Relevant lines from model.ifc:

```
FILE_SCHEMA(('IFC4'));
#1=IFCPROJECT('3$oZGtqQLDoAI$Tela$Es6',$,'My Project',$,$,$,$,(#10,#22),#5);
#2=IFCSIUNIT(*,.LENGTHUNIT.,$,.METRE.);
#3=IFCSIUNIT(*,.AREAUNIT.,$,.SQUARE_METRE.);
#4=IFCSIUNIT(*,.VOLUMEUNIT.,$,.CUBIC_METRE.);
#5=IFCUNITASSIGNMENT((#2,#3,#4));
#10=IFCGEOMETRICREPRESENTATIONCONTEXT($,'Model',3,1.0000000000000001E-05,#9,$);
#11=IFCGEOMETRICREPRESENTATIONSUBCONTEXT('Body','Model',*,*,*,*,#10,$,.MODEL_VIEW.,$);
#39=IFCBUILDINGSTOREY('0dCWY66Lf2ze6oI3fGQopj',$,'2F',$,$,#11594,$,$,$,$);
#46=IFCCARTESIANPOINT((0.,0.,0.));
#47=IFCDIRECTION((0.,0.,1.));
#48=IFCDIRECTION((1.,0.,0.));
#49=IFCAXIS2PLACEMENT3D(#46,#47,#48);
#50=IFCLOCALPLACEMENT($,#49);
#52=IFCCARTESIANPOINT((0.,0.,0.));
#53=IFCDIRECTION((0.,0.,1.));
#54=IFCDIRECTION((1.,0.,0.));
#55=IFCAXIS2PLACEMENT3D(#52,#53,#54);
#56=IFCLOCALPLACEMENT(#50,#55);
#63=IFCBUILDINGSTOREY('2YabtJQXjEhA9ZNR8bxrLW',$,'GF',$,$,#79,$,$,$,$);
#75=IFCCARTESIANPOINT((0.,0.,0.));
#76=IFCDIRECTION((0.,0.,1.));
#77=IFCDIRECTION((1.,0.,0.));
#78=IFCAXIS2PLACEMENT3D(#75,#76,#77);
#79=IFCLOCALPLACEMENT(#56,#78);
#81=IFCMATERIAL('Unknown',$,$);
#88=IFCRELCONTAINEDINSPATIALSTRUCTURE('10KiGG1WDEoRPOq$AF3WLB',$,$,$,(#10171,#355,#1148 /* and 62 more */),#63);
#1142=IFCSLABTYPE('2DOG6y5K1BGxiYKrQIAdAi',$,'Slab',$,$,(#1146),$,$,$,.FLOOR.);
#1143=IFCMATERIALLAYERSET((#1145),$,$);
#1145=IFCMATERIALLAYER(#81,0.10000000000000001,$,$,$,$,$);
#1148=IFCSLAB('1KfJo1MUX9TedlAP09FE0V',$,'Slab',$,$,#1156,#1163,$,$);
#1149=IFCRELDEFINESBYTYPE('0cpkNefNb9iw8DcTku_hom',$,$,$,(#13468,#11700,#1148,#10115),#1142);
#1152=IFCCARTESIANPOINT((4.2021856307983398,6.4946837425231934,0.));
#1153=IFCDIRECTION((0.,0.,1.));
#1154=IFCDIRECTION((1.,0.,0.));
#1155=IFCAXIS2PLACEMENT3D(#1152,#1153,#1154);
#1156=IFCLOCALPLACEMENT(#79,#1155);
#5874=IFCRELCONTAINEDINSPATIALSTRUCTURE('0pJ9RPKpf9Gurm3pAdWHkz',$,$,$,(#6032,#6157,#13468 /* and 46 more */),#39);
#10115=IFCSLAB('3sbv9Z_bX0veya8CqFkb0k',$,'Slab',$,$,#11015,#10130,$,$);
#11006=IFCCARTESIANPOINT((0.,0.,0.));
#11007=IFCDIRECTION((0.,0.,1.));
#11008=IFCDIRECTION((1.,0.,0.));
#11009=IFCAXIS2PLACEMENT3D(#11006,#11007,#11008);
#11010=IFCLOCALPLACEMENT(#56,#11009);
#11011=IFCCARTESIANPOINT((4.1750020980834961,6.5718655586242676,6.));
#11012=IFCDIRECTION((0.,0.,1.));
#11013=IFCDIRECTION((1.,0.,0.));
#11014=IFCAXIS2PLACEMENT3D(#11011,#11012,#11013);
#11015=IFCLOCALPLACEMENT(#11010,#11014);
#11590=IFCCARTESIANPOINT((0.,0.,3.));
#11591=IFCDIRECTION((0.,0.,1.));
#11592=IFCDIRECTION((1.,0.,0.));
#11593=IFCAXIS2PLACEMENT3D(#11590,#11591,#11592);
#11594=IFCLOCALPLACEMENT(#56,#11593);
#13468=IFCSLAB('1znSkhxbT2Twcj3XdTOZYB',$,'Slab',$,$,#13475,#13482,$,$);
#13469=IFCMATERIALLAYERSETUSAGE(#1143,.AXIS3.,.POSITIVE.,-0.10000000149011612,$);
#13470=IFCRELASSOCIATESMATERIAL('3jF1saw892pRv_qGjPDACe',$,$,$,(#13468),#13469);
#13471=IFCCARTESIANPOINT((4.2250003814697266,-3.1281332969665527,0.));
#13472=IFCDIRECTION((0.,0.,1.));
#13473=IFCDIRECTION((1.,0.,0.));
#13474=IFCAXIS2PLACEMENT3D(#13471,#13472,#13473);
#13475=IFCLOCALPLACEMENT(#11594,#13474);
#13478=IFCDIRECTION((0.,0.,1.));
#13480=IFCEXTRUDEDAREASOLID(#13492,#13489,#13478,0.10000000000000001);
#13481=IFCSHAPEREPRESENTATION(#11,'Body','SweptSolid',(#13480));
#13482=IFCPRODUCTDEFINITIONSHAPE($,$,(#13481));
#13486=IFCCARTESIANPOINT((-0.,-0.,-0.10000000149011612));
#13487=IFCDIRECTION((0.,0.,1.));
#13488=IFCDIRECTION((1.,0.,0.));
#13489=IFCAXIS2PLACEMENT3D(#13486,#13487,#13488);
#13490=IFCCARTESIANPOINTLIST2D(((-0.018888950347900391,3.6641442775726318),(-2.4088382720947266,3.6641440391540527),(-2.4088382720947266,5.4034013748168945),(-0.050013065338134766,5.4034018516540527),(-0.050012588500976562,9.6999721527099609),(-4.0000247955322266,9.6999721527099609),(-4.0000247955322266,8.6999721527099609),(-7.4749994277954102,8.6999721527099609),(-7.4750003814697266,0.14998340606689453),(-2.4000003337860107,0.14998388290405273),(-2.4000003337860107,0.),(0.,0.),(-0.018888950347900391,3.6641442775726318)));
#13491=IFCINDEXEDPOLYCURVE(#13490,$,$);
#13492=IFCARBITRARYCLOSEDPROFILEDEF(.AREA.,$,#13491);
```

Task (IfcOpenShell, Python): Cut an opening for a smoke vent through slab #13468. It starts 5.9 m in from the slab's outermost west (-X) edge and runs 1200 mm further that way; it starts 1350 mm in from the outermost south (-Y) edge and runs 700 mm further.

```python
import numpy as np
import ifcopenshell
import ifcopenshell.api.feature
import ifcopenshell.api.geometry
import ifcopenshell.api.root
import ifcopenshell.geom
import ifcopenshell.util.placement
import ifcopenshell.util.representation
import ifcopenshell.util.shape
import ifcopenshell.util.unit

model = ifcopenshell.open("model.ifc")
unit_scale = ifcopenshell.util.unit.calculate_unit_scale(model)
settings = ifcopenshell.geom.settings()


def volume(element):
    """Net volume in cubic metres, openings subtracted."""
    shape = ifcopenshell.geom.create_shape(settings, element)
    return ifcopenshell.util.shape.get_volume(shape.geometry)


slab = model.by_guid("1znSkhxbT2Twcj3XdTOZYB")
before = volume(slab)

# Extent in the slab's own axes, in metres. The edges named are its -X and -Y sides.
slab_shape = ifcopenshell.geom.create_shape(settings, slab)
vertices = ifcopenshell.util.shape.get_vertices(slab_shape.geometry)
x_min, y_min, bottom = vertices.min(axis=0)
top = vertices[:, 2].max()

opening = ifcopenshell.api.root.create_entity(model, ifc_class="IfcOpeningElement", name="Smoke vent opening", predefined_type="OPENING")
context = ifcopenshell.util.representation.get_context(model, "Model", "Body", "MODEL_VIEW")
width, depth = 1.2, 0.7
outline = [(0.0, 0.0), (width, 0.0), (width, depth), (0.0, depth), (0.0, 0.0)]
# Overshoot both faces by 50 mm so the cut is clean.
shape = ifcopenshell.api.geometry.add_slab_representation(
    model, context=context, depth=top - bottom + 0.1, polyline=outline
)
ifcopenshell.api.geometry.assign_representation(model, product=opening, representation=shape)

matrix = ifcopenshell.util.placement.get_local_placement(slab.ObjectPlacement)
matrix[:, 3] = matrix @ np.append(np.array([x_min + 5.9, y_min + 1.35, bottom - 0.05]) / unit_scale, 1.0)
ifcopenshell.api.geometry.edit_object_placement(model, product=opening, matrix=matrix, is_si=False)
ifcopenshell.api.feature.add_feature(model, feature=opening, element=slab)

after = volume(slab)

print(f"slab volume {before:.3f} -> {after:.3f} m3")

model.write("model_v2.ifc")
```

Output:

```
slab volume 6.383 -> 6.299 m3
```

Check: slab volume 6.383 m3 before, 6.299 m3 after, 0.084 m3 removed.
